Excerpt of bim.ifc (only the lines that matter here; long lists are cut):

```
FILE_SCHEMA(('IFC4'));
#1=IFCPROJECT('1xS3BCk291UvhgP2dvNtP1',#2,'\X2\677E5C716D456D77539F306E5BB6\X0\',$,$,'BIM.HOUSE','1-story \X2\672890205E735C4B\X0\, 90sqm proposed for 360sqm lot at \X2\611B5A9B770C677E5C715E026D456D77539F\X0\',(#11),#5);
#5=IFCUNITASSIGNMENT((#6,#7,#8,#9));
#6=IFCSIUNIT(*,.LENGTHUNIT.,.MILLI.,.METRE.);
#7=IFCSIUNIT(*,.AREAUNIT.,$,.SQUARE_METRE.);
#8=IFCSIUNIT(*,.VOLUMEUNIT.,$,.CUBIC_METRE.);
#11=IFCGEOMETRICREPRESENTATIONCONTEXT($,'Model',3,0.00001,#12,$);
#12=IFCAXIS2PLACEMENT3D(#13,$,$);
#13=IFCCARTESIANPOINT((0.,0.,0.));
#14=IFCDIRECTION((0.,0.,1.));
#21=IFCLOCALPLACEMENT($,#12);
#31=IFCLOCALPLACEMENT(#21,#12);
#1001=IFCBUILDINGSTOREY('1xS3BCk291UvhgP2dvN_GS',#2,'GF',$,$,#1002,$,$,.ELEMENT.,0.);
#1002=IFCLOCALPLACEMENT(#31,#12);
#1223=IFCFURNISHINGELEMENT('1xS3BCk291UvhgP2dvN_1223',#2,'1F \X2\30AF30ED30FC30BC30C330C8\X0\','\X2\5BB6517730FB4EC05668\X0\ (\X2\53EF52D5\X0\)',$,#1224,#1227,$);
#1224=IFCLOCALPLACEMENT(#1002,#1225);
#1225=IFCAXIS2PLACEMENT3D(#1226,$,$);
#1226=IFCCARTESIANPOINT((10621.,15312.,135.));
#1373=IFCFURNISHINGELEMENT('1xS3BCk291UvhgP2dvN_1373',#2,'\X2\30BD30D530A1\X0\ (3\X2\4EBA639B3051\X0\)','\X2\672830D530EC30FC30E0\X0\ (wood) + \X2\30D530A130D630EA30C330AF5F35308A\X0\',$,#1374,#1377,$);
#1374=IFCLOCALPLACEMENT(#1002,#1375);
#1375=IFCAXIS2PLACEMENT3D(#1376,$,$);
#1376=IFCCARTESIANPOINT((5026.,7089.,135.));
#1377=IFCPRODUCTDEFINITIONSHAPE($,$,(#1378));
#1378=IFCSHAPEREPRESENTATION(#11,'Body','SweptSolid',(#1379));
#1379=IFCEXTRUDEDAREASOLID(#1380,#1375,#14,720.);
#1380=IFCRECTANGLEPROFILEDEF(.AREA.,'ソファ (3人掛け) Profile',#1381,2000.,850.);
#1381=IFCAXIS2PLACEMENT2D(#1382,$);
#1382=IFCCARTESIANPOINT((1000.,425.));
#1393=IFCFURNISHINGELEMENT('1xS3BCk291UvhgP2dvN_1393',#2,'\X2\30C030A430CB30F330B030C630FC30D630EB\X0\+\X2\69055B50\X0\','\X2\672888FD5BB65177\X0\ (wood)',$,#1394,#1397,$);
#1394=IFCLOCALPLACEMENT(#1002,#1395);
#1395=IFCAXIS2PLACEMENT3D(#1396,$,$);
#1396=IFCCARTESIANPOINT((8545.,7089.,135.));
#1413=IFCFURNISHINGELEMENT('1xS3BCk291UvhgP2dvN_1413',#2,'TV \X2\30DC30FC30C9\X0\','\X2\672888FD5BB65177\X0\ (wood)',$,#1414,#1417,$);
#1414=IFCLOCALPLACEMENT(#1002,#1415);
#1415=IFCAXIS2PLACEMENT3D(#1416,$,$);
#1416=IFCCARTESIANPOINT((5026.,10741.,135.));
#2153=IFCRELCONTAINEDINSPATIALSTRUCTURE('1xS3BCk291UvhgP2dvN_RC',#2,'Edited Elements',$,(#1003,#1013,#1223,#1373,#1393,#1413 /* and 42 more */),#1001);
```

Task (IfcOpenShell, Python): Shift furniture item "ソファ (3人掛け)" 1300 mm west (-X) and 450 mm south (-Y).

```python
import ifcopenshell
import ifcopenshell.api.geometry
import ifcopenshell.util.placement

model = ifcopenshell.open("bim.ifc")

item = model.by_guid("1xS3BCk291UvhgP2dvN_1373")
matrix = ifcopenshell.util.placement.get_local_placement(item.ObjectPlacement)
matrix[0, 3] -= 1300.0
matrix[1, 3] -= 450.0
ifcopenshell.api.geometry.edit_object_placement(model, product=item, matrix=matrix, is_si=False)

print(ifcopenshell.util.placement.get_local_placement(item.ObjectPlacement).round(3) + 0.0)

model.write("bim-out.ifc")
```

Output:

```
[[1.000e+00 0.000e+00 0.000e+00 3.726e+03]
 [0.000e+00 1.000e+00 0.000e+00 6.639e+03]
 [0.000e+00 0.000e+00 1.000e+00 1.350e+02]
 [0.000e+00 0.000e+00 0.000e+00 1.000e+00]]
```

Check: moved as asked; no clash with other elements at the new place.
